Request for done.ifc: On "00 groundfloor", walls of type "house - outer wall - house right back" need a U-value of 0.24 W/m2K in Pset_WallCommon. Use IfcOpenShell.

First a look at what the model holds.

```python
import ifcopenshell
import ifcopenshell.util.element

model = ifcopenshell.open("done.ifc")
print(model.schema)
storey = next(s for s in model.by_type("IfcBuildingStorey") if s.Name == "00 groundfloor")
walls = [e for e in ifcopenshell.util.element.get_decomposition(storey) if e.is_a("IfcWall")]
seen = {}
for e in walls:
    element_type = ifcopenshell.util.element.get_type(e)
    key = (element_type.Name if element_type != e and element_type else None, ifcopenshell.util.element.get_pset(e, "Pset_WallCommon", "ThermalTransmittance"))
    seen[key] = seen.get(key, 0) + 1
for (name, value), count in sorted(seen.items(), key=str):
    print(count, "x", name, "|", value)
```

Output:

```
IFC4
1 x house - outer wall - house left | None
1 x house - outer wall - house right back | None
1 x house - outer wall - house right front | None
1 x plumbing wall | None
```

```python
import ifcopenshell
import ifcopenshell.api.pset
import ifcopenshell.util.element

model = ifcopenshell.open("done.ifc")

storey = next(s for s in model.by_type("IfcBuildingStorey") if s.Name == "00 groundfloor")
walls = [e for e in ifcopenshell.util.element.get_decomposition(storey) if e.is_a("IfcWall")]

count = 0
for e in walls:
    element_type = ifcopenshell.util.element.get_type(e)
    if element_type in (None, e) or element_type.Name != "house - outer wall - house right back":
        continue
    # add_pset returns the element's existing set when there is one.
    pset = ifcopenshell.api.pset.add_pset(model, product=e, name="Pset_WallCommon")
    ifcopenshell.api.pset.edit_pset(model, pset=pset, properties={"ThermalTransmittance": 0.24})
    count += 1

print(count, "walls updated")

model.write("done-out.ifc")
```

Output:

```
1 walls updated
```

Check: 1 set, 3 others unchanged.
